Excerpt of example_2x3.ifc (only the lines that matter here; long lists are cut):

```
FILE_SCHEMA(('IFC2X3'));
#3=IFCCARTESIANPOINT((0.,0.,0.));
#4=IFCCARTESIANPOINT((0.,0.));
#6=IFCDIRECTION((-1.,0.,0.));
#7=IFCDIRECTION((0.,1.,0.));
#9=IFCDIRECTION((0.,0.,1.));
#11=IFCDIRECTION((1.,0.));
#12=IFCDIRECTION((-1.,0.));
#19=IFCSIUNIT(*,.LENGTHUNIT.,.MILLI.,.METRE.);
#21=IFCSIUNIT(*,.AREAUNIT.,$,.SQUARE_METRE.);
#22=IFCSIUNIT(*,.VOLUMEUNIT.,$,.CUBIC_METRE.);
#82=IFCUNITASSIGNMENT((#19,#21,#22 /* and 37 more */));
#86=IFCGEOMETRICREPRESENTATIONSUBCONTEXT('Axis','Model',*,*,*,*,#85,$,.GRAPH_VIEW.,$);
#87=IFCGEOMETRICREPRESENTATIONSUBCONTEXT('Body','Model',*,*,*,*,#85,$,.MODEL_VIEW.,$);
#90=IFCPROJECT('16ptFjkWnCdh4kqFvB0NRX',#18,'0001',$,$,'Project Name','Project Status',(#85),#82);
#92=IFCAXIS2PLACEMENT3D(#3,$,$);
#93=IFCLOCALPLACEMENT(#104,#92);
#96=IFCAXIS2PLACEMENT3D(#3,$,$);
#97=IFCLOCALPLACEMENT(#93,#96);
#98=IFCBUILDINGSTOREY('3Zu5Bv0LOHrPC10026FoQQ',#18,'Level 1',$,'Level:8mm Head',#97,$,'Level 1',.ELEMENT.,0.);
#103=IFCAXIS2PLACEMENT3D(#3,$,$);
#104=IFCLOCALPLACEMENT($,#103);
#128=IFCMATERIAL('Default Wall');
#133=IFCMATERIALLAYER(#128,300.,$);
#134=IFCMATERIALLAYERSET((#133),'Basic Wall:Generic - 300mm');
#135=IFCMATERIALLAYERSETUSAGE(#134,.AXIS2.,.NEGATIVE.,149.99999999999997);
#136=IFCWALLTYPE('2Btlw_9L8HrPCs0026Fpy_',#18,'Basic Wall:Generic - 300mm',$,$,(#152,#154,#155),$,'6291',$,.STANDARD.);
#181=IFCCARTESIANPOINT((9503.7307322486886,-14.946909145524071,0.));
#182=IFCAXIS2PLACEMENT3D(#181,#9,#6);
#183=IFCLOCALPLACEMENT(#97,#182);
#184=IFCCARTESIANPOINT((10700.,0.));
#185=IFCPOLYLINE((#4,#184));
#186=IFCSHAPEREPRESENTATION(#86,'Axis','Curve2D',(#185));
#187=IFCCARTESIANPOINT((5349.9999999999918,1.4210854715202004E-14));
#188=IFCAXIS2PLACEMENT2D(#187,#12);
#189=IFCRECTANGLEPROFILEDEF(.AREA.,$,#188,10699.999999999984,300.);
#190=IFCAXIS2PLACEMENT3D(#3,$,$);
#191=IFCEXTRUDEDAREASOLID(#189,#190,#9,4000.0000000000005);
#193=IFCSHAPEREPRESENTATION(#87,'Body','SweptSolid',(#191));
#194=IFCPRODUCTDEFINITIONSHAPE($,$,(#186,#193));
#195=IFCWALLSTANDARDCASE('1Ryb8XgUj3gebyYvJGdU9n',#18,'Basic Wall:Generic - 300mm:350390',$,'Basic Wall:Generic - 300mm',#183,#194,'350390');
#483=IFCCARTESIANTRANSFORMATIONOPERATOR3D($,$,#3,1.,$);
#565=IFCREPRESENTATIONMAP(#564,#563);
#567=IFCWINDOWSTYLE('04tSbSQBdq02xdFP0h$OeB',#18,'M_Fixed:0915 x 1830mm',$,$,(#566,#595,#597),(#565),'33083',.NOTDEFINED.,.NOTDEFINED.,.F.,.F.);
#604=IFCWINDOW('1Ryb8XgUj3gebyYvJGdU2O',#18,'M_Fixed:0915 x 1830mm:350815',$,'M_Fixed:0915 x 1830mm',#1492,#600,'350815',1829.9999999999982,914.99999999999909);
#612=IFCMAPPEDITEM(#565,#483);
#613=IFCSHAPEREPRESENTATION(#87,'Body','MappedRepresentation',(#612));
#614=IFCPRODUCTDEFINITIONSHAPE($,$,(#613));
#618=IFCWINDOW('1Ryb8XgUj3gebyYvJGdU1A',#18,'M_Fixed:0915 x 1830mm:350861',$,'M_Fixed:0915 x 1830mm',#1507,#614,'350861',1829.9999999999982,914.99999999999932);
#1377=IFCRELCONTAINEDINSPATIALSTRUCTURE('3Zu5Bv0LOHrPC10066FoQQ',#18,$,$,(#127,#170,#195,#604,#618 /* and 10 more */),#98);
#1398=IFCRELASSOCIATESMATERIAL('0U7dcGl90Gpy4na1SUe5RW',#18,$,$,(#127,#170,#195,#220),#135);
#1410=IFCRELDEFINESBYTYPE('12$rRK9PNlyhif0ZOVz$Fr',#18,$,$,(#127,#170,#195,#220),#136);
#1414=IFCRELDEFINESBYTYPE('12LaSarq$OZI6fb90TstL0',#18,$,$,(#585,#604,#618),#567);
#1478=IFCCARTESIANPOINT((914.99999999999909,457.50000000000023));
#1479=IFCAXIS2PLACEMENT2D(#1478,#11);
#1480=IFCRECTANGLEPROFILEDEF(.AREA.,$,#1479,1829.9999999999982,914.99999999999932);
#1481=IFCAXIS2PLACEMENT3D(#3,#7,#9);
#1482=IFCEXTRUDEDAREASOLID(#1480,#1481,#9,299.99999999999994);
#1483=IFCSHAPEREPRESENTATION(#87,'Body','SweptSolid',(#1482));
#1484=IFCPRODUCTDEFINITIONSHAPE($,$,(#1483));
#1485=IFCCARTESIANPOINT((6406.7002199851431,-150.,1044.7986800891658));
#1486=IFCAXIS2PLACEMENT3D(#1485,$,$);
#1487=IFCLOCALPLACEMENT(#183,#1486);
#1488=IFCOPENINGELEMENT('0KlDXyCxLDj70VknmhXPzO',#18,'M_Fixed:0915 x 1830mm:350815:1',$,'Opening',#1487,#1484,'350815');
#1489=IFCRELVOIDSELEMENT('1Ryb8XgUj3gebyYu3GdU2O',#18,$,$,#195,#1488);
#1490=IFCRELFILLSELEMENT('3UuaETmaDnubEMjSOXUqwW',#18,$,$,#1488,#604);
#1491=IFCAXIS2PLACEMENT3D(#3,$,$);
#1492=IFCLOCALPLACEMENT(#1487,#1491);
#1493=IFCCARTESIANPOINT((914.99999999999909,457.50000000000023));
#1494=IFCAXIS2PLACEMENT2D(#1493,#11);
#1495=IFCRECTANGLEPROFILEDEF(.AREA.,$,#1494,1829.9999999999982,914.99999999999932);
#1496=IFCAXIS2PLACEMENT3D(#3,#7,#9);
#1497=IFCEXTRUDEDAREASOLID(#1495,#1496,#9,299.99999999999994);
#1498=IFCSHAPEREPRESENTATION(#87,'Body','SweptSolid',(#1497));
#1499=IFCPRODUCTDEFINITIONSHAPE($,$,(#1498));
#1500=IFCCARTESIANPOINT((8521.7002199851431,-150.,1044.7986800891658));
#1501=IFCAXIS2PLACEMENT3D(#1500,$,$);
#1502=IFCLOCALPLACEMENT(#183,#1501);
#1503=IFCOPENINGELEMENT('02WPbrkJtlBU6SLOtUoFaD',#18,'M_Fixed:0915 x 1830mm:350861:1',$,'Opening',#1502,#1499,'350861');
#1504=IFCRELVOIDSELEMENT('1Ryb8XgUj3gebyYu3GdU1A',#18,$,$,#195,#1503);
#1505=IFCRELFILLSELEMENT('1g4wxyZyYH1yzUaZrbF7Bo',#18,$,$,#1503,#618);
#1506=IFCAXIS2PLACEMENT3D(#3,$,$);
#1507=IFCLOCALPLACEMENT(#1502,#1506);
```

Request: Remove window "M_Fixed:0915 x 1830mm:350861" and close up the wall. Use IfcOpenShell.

```python
import ifcopenshell
import ifcopenshell.api.feature
import ifcopenshell.api.root
import ifcopenshell.geom
import ifcopenshell.util.shape

model = ifcopenshell.open("example_2x3.ifc")
settings = ifcopenshell.geom.settings()


def volume(element):
    """Net volume in cubic metres, openings subtracted."""
    shape = ifcopenshell.geom.create_shape(settings, element)
    return ifcopenshell.util.shape.get_volume(shape.geometry)


window = model.by_guid("1Ryb8XgUj3gebyYvJGdU1A")
opening = window.FillsVoids[0].RelatingOpeningElement
wall = opening.VoidsElements[0].RelatingBuildingElement
before = volume(wall)

ifcopenshell.api.root.remove_product(model, product=window)
ifcopenshell.api.feature.remove_feature(model, feature=opening)

after = volume(wall)

print(f"wall volume {before:.3f} -> {after:.3f} m3")

model.write("example_2x3-out.ifc")
```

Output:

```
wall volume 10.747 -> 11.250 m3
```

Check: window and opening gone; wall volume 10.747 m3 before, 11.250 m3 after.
